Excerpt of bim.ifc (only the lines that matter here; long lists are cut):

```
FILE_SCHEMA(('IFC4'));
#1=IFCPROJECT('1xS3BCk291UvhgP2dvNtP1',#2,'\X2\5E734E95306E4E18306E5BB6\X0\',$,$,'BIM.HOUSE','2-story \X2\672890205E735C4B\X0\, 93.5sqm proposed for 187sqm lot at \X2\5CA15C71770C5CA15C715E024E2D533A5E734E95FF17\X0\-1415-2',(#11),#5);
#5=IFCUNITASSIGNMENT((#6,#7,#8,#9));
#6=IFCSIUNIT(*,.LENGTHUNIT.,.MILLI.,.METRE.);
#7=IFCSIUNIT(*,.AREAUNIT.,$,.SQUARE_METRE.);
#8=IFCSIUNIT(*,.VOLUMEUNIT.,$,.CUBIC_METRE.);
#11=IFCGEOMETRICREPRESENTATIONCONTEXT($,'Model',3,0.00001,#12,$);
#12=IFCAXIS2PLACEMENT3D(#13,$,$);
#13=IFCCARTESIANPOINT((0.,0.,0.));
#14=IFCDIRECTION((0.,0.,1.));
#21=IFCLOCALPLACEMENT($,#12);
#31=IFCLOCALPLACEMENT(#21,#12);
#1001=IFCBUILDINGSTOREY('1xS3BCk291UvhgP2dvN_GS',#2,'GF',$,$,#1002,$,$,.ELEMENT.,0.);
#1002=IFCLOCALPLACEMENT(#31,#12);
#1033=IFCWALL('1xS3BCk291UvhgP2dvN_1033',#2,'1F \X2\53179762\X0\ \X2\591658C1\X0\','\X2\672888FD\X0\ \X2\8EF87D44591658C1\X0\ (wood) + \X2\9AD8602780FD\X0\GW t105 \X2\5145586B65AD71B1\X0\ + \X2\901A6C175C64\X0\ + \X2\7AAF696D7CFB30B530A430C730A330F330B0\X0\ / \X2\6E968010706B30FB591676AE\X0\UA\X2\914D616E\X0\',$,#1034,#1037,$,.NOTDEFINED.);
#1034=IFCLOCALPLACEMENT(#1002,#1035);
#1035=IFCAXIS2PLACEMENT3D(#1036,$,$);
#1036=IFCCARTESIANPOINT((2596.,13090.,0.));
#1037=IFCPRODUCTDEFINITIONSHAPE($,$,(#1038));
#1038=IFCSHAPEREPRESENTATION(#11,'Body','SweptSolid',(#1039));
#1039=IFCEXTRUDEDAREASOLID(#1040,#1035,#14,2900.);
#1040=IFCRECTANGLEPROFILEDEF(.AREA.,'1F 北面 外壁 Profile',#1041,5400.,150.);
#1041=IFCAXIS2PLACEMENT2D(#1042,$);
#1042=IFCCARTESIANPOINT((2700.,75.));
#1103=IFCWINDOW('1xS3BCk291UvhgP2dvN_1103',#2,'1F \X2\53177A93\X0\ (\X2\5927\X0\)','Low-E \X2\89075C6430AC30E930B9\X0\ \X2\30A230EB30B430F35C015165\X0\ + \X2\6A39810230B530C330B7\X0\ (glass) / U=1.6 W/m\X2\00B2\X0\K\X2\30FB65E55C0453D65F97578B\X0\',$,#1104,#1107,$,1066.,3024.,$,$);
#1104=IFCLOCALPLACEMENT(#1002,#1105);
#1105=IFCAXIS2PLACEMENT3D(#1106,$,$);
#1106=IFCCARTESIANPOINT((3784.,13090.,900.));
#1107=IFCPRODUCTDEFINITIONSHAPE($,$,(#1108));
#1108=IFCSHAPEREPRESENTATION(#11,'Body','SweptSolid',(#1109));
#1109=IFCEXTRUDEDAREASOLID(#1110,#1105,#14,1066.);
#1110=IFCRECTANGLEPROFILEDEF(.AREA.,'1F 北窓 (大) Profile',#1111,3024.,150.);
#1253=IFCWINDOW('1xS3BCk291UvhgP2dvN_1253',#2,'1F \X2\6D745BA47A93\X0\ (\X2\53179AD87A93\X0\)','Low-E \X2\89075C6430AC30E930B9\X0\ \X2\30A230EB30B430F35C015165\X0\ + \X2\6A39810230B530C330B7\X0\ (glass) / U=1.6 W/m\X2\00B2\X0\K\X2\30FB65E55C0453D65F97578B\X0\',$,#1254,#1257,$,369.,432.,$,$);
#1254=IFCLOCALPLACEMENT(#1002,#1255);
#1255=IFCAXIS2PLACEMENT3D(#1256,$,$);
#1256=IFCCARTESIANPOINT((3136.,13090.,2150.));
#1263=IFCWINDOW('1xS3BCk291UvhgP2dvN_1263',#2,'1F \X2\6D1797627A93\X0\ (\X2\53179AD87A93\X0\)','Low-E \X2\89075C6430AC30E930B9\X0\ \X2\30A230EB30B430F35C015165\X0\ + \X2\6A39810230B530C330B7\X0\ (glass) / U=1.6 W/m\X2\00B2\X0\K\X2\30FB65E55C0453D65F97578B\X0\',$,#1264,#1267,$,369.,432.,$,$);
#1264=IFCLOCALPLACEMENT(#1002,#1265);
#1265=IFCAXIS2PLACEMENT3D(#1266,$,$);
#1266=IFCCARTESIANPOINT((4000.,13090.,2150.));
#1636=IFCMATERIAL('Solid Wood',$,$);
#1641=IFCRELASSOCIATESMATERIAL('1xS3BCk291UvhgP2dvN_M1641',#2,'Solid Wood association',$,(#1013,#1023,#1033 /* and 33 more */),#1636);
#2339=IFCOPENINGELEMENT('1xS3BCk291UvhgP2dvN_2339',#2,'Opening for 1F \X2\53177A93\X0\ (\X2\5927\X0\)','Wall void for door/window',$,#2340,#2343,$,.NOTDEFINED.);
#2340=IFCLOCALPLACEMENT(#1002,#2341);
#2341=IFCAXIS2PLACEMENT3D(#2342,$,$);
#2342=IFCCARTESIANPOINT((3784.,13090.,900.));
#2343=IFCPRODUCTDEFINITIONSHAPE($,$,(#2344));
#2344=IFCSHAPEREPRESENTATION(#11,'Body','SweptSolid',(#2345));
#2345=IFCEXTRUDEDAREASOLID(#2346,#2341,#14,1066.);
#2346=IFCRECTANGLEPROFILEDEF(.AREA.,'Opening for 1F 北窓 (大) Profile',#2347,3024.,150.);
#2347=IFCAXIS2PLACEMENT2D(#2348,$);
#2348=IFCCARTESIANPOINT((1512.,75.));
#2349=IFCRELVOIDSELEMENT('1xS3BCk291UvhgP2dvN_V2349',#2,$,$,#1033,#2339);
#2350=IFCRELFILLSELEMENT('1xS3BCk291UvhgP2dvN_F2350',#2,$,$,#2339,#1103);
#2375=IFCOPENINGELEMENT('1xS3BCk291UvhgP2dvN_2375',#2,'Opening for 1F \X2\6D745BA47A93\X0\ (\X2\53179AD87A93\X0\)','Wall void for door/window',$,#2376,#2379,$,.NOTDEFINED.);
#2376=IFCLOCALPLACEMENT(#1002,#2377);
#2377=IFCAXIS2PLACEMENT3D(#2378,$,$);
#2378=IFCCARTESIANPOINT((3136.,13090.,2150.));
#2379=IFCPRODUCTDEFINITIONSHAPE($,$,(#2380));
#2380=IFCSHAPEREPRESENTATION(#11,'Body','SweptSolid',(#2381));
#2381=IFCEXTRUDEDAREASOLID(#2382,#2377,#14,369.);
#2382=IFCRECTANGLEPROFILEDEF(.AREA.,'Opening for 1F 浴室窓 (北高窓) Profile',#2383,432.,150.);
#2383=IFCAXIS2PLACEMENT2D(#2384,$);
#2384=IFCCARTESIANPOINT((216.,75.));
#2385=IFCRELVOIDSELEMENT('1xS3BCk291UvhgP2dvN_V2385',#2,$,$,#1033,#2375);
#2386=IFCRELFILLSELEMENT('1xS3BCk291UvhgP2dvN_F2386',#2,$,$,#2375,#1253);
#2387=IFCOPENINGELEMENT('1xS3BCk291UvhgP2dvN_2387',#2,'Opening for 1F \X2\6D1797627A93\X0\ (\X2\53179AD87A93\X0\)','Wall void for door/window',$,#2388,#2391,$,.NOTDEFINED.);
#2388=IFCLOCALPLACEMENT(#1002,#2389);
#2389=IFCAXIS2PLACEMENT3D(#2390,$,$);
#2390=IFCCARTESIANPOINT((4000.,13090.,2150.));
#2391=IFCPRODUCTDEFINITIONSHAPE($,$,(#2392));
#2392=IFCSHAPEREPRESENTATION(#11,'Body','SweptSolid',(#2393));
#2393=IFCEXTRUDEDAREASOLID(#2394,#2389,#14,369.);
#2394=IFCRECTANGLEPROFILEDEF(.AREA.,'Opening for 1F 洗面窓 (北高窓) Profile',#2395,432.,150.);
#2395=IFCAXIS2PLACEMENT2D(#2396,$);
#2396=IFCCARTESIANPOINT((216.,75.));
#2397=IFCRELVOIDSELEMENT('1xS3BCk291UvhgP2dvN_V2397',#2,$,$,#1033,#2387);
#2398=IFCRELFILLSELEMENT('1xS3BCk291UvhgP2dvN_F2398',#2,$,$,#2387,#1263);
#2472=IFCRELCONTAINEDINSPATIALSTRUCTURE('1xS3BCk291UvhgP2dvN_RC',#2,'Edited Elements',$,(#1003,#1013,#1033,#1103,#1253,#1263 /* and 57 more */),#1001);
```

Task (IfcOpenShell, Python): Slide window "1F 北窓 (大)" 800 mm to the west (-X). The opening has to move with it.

```python
import ifcopenshell
import ifcopenshell.api.geometry
import ifcopenshell.util.placement
import ifcopenshell.util.unit

model = ifcopenshell.open("bim.ifc")
unit_scale = ifcopenshell.util.unit.calculate_unit_scale(model)

window = model.by_guid("1xS3BCk291UvhgP2dvN_1103")
opening = window.FillsVoids[0].RelatingOpeningElement
wall = opening.VoidsElements[0].RelatingBuildingElement

wall_matrix = ifcopenshell.util.placement.get_local_placement(wall.ObjectPlacement)
shift = wall_matrix[:3, 0] * -0.8 / unit_scale
before = ifcopenshell.util.placement.get_local_placement(window.ObjectPlacement)[:3, 3].copy()

# The window is not placed relative to its opening, so move both.
for product in (opening, window):
    matrix = ifcopenshell.util.placement.get_local_placement(product.ObjectPlacement)
    matrix[:3, 3] += shift
    ifcopenshell.api.geometry.edit_object_placement(model, product=product, matrix=matrix, is_si=False)

after = ifcopenshell.util.placement.get_local_placement(window.ObjectPlacement)[:3, 3]
print("window moved by", (after - before).round(3) + 0.0)

model.write("bim_rev.ifc")
```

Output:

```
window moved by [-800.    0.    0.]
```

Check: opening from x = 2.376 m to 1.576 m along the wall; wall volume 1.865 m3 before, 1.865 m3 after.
